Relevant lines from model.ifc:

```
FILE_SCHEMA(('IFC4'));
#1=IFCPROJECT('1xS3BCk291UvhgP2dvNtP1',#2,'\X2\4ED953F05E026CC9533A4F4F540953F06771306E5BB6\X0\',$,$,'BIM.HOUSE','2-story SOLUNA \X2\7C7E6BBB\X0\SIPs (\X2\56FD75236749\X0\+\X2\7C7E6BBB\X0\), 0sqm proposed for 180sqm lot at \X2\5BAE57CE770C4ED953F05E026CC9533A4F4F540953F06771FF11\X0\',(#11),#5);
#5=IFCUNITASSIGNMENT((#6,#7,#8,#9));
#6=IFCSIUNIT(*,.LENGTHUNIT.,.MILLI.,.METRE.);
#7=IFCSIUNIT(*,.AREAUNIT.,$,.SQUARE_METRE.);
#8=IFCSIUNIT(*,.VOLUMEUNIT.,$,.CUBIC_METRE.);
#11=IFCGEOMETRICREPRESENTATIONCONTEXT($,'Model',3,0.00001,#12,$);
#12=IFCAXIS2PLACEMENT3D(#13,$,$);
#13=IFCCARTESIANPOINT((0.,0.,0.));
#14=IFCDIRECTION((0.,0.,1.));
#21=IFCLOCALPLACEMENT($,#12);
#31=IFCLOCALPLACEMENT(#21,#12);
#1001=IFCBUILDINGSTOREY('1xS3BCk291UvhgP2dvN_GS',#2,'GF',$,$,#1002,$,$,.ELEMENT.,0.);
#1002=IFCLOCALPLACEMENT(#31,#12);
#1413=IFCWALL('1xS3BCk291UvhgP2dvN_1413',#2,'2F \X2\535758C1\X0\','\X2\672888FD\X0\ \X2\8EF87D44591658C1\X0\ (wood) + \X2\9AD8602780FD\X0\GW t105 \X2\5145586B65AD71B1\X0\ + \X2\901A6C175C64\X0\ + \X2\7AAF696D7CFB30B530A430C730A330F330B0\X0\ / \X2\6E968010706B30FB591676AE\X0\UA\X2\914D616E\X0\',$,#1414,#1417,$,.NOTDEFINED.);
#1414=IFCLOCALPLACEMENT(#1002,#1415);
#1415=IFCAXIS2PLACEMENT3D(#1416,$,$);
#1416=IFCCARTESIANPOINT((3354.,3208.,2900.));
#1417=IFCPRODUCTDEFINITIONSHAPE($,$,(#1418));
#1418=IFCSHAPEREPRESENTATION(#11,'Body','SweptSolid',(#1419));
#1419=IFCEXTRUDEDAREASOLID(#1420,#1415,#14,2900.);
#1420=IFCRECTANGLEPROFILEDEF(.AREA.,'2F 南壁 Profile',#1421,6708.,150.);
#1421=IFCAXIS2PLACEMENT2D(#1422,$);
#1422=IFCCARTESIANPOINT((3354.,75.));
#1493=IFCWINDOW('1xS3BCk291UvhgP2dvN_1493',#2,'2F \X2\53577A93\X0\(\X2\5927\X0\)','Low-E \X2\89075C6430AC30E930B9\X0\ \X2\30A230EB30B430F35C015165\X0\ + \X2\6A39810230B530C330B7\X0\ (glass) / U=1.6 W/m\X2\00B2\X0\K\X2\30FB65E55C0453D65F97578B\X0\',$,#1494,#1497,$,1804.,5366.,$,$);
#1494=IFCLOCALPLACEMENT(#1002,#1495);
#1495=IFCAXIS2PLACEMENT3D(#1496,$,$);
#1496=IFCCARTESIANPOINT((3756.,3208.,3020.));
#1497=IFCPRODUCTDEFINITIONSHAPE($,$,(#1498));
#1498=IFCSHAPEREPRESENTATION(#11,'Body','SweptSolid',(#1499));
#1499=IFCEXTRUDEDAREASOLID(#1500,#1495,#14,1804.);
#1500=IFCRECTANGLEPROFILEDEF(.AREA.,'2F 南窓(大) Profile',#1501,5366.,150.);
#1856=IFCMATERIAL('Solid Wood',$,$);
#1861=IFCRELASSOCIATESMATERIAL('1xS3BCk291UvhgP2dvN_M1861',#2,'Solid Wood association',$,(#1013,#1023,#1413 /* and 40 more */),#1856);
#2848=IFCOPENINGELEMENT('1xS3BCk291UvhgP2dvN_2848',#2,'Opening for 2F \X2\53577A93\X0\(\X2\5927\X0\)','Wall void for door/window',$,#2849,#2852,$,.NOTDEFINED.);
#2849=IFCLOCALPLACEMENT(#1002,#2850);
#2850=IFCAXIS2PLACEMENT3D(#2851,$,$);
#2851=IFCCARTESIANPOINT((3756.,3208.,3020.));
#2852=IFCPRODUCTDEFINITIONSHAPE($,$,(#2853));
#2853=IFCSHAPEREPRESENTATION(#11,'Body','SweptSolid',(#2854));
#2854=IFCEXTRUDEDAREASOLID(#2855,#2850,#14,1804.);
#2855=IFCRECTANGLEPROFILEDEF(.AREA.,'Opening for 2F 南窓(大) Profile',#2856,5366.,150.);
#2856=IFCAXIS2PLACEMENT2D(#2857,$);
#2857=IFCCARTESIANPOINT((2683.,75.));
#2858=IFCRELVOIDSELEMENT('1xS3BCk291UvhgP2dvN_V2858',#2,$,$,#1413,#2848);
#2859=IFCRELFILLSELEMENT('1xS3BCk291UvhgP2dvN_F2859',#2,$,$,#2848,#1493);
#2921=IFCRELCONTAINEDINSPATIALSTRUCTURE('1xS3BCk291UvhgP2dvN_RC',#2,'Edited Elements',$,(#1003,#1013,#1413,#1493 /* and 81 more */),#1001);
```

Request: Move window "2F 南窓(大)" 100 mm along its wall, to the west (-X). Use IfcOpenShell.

```python
import ifcopenshell
import ifcopenshell.api.geometry
import ifcopenshell.util.placement
import ifcopenshell.util.unit

model = ifcopenshell.open("model.ifc")
unit_scale = ifcopenshell.util.unit.calculate_unit_scale(model)

window = model.by_id(1493)
opening = window.FillsVoids[0].RelatingOpeningElement
wall = opening.VoidsElements[0].RelatingBuildingElement

wall_matrix = ifcopenshell.util.placement.get_local_placement(wall.ObjectPlacement)
shift = wall_matrix[:3, 0] * -0.1 / unit_scale
before = ifcopenshell.util.placement.get_local_placement(window.ObjectPlacement)[:3, 3].copy()

# The window is not placed relative to its opening, so move both.
for product in (opening, window):
    matrix = ifcopenshell.util.placement.get_local_placement(product.ObjectPlacement)
    matrix[:3, 3] += shift
    ifcopenshell.api.geometry.edit_object_placement(model, product=product, matrix=matrix, is_si=False)

after = ifcopenshell.util.placement.get_local_placement(window.ObjectPlacement)[:3, 3]
print("window moved by", (after - before).round(3) + 0.0)

model.write("model-out.ifc")
```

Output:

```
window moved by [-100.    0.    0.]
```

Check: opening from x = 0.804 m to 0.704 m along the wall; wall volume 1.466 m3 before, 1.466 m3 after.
